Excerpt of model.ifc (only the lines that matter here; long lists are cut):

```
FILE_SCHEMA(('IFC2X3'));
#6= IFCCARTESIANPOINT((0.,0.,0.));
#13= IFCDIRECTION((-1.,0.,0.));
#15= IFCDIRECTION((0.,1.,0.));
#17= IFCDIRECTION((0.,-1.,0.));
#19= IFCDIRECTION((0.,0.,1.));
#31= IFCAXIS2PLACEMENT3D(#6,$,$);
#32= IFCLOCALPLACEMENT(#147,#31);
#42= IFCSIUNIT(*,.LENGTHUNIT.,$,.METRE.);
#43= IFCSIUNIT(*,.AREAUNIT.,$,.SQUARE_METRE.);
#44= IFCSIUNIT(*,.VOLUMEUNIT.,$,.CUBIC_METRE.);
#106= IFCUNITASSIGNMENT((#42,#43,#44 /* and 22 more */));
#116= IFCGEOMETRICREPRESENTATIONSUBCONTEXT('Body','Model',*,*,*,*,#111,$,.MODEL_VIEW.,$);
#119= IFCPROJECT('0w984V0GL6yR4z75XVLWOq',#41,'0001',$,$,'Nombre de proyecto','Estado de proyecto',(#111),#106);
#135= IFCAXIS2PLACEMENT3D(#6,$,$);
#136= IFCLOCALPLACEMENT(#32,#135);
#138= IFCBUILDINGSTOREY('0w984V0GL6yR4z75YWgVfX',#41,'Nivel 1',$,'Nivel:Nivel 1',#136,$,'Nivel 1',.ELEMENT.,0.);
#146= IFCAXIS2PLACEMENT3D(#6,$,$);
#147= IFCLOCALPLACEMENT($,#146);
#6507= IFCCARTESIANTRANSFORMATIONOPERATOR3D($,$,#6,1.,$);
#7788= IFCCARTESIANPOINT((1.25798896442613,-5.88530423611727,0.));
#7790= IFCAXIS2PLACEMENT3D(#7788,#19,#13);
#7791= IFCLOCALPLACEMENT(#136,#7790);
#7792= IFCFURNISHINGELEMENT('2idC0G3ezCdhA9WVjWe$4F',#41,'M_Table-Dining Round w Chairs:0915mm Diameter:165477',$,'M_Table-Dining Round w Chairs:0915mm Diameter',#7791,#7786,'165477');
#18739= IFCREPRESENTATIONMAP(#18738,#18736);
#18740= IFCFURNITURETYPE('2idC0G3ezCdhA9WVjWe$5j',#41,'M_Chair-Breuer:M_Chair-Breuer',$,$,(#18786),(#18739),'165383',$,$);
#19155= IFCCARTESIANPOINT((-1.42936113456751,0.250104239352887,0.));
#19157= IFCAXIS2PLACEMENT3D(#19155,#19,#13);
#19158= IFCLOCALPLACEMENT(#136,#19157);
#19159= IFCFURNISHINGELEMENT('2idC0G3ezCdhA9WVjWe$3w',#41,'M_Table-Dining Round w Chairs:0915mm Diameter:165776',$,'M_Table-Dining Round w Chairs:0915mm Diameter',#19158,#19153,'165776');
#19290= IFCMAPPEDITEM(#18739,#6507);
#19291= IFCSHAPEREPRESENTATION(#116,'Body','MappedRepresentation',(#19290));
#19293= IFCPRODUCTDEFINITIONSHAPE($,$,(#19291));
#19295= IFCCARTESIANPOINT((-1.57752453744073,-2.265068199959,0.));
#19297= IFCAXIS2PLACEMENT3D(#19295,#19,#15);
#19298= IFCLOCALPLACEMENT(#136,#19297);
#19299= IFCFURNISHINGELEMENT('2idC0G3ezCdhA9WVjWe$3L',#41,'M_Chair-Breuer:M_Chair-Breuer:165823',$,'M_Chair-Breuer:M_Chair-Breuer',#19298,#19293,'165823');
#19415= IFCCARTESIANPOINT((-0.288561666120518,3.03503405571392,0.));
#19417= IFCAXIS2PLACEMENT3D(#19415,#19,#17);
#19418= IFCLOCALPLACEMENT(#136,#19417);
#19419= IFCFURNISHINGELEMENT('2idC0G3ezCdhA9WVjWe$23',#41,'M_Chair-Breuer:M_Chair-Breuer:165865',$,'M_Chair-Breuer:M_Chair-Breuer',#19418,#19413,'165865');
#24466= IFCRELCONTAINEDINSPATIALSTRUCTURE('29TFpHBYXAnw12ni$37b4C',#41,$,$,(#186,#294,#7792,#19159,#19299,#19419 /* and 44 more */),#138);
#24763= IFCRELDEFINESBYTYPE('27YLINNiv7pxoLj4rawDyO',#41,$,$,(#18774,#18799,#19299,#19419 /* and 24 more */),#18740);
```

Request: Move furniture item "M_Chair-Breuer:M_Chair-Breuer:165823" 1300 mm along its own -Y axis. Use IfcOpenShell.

```python
import ifcopenshell
import ifcopenshell.api.geometry
import ifcopenshell.util.placement
import ifcopenshell.util.unit

model = ifcopenshell.open("model.ifc")
unit_scale = ifcopenshell.util.unit.calculate_unit_scale(model)

item = model.by_id(19299)
matrix = ifcopenshell.util.placement.get_local_placement(item.ObjectPlacement)
matrix[:3, 3] -= matrix[:3, 1] * 1.3 / unit_scale
ifcopenshell.api.geometry.edit_object_placement(model, product=item, matrix=matrix, is_si=False)

print(ifcopenshell.util.placement.get_local_placement(item.ObjectPlacement).round(3) + 0.0)

model.write("model_updated.ifc")
```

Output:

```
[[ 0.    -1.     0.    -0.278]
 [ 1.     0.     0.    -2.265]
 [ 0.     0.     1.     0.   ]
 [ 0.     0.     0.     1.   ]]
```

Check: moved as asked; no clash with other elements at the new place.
